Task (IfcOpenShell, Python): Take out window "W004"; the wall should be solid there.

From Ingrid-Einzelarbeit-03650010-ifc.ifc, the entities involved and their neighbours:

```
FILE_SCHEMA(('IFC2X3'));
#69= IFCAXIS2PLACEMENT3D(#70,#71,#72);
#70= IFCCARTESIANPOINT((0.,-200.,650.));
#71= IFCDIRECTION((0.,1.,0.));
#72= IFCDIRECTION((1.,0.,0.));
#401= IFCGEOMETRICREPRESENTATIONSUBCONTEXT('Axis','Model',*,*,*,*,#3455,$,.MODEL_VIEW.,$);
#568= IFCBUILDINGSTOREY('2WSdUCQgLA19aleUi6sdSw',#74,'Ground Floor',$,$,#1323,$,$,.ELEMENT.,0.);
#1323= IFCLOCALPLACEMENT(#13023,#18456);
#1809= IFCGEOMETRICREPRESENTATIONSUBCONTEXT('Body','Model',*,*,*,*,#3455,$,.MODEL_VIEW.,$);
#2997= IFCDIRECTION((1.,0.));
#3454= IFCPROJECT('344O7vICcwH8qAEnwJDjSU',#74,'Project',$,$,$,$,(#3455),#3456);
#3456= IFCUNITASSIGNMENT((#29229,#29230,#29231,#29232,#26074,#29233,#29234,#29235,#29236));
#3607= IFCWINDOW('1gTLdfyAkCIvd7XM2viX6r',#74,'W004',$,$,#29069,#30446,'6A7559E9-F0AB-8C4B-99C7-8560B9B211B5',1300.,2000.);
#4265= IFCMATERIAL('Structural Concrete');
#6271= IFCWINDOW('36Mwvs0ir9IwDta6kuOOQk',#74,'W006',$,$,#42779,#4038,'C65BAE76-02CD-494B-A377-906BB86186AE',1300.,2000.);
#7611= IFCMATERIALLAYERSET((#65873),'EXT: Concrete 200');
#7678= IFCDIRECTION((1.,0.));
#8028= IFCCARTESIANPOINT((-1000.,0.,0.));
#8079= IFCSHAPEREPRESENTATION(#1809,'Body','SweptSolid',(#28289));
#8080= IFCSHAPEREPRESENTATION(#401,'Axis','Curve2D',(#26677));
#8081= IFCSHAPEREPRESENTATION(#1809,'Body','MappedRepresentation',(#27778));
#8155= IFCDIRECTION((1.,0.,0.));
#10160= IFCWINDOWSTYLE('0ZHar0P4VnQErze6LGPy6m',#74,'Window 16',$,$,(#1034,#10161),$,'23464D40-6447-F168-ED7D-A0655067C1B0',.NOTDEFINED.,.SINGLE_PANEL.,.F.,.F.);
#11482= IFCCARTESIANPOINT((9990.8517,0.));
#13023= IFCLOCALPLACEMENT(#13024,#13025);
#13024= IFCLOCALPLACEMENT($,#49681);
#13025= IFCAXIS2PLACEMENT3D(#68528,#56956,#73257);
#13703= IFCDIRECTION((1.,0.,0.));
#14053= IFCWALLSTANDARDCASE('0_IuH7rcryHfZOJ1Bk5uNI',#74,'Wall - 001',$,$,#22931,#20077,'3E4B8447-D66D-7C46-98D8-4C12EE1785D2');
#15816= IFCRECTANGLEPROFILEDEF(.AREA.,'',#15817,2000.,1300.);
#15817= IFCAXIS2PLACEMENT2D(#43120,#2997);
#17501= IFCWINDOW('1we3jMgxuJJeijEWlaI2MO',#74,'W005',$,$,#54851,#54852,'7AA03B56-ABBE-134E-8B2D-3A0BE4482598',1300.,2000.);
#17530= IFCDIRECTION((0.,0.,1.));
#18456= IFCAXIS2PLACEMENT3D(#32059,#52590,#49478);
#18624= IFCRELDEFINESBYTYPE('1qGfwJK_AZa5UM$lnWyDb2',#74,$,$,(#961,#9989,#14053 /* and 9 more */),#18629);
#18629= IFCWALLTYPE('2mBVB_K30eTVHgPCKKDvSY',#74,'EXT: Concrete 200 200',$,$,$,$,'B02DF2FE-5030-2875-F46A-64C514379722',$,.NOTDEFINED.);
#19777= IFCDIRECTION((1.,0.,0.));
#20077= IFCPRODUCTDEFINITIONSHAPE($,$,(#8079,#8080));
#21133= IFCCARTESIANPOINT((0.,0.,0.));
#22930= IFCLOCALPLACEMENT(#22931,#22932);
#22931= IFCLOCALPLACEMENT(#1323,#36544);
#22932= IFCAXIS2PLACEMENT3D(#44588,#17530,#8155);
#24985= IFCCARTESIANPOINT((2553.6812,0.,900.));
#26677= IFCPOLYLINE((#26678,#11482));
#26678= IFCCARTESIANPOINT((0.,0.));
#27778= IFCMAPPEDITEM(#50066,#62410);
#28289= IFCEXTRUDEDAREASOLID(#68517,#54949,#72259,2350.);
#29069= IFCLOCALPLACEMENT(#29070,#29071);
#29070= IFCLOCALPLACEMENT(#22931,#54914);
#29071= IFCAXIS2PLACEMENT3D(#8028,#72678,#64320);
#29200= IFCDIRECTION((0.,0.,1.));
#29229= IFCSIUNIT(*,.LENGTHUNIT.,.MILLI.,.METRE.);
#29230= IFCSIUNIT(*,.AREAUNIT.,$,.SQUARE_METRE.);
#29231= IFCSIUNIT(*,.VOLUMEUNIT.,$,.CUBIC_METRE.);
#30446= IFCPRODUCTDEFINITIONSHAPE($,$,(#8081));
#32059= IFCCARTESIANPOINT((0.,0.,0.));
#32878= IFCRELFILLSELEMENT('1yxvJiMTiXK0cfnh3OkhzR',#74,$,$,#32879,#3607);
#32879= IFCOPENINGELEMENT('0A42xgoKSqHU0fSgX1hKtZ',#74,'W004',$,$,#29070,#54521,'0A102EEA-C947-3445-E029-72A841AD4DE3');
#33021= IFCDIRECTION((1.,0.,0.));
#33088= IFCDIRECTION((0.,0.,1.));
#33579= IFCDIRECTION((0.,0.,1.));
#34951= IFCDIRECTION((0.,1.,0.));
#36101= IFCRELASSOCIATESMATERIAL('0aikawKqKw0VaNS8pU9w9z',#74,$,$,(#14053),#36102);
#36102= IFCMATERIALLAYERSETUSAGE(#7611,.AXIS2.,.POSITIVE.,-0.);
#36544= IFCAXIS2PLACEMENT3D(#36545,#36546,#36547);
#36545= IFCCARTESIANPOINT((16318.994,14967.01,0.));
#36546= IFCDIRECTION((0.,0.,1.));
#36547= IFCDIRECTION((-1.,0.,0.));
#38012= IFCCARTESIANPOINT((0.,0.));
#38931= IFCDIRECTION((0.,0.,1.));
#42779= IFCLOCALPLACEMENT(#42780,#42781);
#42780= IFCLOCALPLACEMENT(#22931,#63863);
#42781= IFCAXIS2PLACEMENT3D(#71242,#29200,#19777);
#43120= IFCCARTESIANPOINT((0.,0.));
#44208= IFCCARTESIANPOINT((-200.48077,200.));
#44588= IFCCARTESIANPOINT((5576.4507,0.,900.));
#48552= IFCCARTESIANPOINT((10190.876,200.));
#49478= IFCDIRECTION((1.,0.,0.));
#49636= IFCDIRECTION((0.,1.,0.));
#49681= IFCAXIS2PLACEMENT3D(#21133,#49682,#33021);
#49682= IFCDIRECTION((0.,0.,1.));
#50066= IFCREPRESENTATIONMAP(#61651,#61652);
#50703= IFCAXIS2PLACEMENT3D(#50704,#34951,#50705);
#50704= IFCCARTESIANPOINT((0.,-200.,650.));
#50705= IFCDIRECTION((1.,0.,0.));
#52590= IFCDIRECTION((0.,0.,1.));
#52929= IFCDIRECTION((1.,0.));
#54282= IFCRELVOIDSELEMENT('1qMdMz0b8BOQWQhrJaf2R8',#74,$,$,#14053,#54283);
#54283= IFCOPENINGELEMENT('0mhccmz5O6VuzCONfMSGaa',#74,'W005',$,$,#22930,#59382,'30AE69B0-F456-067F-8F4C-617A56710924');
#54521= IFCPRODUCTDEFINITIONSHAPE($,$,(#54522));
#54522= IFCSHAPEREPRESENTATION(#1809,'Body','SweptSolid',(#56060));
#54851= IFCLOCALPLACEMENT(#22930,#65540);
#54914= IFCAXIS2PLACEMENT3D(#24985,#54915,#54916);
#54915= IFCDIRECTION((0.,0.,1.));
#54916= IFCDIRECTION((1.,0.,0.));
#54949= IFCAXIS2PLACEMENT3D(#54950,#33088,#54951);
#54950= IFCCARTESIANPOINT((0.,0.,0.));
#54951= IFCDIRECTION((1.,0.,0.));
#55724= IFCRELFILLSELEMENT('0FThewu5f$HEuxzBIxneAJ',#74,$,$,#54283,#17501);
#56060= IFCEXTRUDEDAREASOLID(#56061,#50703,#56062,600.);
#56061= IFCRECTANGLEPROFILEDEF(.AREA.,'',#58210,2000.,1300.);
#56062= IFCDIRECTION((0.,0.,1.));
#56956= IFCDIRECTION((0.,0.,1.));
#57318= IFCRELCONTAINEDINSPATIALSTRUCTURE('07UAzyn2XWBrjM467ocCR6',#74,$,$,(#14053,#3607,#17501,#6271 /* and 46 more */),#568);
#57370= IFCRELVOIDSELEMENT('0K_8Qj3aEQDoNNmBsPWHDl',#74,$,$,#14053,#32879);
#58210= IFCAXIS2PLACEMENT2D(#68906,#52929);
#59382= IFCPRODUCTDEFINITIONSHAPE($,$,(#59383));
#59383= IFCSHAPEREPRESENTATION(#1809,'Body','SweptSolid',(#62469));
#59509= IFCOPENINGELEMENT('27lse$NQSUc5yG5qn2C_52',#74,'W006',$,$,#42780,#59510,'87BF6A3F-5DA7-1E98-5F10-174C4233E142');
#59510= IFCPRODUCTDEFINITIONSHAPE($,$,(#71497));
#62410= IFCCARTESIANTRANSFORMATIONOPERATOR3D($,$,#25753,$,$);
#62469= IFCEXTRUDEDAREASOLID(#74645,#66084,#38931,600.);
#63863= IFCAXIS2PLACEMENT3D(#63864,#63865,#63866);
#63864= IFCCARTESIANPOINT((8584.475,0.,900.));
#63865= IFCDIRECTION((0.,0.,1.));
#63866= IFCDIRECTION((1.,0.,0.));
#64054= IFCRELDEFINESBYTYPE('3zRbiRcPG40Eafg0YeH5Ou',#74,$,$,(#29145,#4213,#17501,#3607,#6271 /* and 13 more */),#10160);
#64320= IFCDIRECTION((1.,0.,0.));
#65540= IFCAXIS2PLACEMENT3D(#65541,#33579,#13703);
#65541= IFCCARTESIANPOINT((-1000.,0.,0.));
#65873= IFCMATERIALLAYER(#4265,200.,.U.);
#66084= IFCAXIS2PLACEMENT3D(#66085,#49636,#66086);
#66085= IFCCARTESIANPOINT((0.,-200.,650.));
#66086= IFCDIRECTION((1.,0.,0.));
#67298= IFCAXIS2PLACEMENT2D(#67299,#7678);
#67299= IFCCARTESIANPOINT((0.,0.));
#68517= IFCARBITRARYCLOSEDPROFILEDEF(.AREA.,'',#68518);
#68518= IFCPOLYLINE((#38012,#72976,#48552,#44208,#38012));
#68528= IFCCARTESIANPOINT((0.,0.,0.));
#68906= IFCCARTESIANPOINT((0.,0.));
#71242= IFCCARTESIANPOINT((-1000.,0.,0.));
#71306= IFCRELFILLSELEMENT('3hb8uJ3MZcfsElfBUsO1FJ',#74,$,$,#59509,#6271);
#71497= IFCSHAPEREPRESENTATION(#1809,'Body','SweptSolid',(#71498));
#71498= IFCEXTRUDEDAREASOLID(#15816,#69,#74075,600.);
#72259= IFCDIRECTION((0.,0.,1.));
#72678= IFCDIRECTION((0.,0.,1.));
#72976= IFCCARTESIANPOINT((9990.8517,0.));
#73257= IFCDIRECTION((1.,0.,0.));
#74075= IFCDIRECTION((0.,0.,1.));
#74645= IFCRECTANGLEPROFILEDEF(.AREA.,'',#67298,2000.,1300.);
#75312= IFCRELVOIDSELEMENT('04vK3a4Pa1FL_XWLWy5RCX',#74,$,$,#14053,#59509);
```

```python
import ifcopenshell
import ifcopenshell.api.feature
import ifcopenshell.api.root
import ifcopenshell.geom
import ifcopenshell.util.shape

model = ifcopenshell.open("Ingrid-Einzelarbeit-03650010-ifc.ifc")
settings = ifcopenshell.geom.settings()


def volume(element):
    """Net volume in cubic metres, openings subtracted."""
    shape = ifcopenshell.geom.create_shape(settings, element)
    return ifcopenshell.util.shape.get_volume(shape.geometry)


window = model.by_guid("1gTLdfyAkCIvd7XM2viX6r")
opening = window.FillsVoids[0].RelatingOpeningElement
wall = opening.VoidsElements[0].RelatingBuildingElement
before = volume(wall)

ifcopenshell.api.root.remove_product(model, product=window)
ifcopenshell.api.feature.remove_feature(model, feature=opening)

after = volume(wall)

print(f"wall volume {before:.3f} -> {after:.3f} m3")

model.write("Ingrid-Einzelarbeit-03650010-ifc-out.ifc")
```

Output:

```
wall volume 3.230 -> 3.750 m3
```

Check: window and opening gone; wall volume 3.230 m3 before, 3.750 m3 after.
